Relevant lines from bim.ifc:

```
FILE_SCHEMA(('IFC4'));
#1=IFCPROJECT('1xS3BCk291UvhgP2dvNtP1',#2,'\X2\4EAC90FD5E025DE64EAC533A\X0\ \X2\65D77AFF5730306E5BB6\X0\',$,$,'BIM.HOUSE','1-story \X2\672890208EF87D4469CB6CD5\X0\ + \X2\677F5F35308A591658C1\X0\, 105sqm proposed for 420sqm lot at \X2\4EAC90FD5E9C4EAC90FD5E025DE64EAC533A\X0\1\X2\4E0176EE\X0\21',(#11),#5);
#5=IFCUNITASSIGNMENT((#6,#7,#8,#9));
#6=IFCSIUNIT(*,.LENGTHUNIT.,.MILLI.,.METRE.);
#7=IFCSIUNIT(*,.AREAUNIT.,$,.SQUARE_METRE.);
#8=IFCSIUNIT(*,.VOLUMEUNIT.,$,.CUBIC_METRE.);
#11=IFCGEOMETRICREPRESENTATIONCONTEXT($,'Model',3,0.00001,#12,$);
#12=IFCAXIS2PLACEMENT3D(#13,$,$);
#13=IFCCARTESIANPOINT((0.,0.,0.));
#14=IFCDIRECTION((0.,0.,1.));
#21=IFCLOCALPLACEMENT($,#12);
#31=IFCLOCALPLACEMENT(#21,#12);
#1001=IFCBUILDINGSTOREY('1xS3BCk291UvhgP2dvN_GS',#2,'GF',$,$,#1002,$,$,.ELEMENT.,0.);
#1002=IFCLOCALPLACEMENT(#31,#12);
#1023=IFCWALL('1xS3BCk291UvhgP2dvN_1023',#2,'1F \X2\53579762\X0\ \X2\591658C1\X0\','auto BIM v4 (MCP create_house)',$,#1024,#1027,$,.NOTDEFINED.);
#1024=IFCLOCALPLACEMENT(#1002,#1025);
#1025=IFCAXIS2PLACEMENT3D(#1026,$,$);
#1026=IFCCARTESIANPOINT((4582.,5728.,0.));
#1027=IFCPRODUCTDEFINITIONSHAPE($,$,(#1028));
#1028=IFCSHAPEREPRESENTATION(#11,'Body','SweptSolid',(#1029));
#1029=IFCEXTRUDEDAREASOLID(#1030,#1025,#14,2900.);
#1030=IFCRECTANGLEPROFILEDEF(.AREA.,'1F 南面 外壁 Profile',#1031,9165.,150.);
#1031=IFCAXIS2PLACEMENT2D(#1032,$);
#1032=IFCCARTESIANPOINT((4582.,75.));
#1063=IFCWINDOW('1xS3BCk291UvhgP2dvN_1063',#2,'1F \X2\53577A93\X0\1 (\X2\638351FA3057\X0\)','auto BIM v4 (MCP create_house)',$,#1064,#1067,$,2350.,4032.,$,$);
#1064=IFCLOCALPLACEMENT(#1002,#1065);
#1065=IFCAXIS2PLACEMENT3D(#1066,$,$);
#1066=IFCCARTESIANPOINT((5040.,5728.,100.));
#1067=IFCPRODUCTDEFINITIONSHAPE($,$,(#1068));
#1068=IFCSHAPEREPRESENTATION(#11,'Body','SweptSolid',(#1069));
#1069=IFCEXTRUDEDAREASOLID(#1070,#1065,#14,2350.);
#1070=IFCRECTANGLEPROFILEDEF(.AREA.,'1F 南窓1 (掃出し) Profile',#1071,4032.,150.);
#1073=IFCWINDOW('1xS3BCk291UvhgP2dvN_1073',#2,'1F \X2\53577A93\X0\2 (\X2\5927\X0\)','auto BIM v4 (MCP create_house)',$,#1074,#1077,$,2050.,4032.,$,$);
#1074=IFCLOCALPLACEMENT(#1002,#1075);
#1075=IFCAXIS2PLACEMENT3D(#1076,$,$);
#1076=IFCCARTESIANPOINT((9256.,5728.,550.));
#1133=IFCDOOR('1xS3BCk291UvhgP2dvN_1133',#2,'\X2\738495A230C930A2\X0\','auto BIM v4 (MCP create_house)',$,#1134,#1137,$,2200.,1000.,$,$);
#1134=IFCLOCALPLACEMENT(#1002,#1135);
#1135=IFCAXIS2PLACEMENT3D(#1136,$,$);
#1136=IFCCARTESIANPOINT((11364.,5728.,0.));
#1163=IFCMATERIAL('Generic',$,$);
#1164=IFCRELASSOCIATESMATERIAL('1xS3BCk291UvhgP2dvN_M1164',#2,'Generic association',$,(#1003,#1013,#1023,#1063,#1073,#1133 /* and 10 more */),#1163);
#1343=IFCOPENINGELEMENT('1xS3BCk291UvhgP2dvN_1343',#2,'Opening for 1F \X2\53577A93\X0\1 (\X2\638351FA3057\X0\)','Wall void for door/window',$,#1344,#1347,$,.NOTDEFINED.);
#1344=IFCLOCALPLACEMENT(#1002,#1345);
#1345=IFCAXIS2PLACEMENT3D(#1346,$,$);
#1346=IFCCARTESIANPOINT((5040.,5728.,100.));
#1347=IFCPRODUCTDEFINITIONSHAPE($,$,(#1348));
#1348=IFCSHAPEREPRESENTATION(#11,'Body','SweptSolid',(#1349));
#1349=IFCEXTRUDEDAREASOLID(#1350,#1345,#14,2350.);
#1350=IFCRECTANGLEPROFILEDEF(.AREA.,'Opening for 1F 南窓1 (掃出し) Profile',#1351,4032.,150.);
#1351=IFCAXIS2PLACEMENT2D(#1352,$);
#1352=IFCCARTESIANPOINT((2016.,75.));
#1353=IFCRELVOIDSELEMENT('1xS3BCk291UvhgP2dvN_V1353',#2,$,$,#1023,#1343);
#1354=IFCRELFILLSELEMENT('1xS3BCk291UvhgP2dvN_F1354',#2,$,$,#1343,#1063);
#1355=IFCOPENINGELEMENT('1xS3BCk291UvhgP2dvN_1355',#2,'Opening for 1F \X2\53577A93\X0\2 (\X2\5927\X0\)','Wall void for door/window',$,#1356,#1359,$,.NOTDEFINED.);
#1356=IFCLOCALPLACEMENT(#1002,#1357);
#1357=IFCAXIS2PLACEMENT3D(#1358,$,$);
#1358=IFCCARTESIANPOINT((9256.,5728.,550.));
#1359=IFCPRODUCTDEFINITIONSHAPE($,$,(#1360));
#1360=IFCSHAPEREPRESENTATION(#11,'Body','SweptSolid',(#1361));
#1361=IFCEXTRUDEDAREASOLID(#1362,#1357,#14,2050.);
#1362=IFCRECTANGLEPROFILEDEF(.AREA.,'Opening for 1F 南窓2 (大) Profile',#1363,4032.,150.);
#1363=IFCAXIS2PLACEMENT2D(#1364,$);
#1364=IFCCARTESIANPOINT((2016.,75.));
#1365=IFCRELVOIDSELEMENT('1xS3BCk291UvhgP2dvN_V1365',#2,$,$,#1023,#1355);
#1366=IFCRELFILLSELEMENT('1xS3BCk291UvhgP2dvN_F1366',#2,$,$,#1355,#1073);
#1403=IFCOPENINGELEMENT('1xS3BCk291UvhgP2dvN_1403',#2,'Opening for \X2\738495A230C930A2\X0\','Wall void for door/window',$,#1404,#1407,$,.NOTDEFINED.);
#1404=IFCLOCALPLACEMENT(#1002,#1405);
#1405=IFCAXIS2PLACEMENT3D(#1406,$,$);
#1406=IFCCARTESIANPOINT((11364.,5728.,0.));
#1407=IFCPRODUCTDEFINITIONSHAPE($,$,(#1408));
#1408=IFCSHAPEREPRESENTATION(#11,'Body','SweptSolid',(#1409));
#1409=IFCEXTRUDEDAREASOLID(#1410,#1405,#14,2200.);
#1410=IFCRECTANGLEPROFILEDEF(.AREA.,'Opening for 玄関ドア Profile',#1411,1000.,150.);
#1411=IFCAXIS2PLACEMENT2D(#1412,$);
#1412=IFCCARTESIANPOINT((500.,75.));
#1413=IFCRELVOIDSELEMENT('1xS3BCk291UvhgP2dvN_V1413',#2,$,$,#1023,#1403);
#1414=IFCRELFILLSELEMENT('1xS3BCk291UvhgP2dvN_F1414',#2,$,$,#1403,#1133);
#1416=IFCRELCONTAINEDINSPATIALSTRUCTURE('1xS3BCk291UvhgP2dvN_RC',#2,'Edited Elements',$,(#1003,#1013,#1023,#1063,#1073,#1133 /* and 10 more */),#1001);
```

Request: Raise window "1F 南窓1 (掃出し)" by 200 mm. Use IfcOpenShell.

```python
import numpy as np
import ifcopenshell
import ifcopenshell.api.geometry
import ifcopenshell.util.placement
import ifcopenshell.util.unit

model = ifcopenshell.open("bim.ifc")
unit_scale = ifcopenshell.util.unit.calculate_unit_scale(model)

window = model.by_guid("1xS3BCk291UvhgP2dvN_1063")
opening = window.FillsVoids[0].RelatingOpeningElement
dz = 200.0

shift = np.array([0.0, 0.0, dz])
# The window is not placed relative to its opening, so move both.
for product in (opening, window):
    matrix = ifcopenshell.util.placement.get_local_placement(product.ObjectPlacement)
    matrix[:3, 3] += shift
    ifcopenshell.api.geometry.edit_object_placement(model, product=product, matrix=matrix, is_si=False)

print(f"moved by {dz * unit_scale:+.3f} m")

model.write("bim_updated.ifc")
```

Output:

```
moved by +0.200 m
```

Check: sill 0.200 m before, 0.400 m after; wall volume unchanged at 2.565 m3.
